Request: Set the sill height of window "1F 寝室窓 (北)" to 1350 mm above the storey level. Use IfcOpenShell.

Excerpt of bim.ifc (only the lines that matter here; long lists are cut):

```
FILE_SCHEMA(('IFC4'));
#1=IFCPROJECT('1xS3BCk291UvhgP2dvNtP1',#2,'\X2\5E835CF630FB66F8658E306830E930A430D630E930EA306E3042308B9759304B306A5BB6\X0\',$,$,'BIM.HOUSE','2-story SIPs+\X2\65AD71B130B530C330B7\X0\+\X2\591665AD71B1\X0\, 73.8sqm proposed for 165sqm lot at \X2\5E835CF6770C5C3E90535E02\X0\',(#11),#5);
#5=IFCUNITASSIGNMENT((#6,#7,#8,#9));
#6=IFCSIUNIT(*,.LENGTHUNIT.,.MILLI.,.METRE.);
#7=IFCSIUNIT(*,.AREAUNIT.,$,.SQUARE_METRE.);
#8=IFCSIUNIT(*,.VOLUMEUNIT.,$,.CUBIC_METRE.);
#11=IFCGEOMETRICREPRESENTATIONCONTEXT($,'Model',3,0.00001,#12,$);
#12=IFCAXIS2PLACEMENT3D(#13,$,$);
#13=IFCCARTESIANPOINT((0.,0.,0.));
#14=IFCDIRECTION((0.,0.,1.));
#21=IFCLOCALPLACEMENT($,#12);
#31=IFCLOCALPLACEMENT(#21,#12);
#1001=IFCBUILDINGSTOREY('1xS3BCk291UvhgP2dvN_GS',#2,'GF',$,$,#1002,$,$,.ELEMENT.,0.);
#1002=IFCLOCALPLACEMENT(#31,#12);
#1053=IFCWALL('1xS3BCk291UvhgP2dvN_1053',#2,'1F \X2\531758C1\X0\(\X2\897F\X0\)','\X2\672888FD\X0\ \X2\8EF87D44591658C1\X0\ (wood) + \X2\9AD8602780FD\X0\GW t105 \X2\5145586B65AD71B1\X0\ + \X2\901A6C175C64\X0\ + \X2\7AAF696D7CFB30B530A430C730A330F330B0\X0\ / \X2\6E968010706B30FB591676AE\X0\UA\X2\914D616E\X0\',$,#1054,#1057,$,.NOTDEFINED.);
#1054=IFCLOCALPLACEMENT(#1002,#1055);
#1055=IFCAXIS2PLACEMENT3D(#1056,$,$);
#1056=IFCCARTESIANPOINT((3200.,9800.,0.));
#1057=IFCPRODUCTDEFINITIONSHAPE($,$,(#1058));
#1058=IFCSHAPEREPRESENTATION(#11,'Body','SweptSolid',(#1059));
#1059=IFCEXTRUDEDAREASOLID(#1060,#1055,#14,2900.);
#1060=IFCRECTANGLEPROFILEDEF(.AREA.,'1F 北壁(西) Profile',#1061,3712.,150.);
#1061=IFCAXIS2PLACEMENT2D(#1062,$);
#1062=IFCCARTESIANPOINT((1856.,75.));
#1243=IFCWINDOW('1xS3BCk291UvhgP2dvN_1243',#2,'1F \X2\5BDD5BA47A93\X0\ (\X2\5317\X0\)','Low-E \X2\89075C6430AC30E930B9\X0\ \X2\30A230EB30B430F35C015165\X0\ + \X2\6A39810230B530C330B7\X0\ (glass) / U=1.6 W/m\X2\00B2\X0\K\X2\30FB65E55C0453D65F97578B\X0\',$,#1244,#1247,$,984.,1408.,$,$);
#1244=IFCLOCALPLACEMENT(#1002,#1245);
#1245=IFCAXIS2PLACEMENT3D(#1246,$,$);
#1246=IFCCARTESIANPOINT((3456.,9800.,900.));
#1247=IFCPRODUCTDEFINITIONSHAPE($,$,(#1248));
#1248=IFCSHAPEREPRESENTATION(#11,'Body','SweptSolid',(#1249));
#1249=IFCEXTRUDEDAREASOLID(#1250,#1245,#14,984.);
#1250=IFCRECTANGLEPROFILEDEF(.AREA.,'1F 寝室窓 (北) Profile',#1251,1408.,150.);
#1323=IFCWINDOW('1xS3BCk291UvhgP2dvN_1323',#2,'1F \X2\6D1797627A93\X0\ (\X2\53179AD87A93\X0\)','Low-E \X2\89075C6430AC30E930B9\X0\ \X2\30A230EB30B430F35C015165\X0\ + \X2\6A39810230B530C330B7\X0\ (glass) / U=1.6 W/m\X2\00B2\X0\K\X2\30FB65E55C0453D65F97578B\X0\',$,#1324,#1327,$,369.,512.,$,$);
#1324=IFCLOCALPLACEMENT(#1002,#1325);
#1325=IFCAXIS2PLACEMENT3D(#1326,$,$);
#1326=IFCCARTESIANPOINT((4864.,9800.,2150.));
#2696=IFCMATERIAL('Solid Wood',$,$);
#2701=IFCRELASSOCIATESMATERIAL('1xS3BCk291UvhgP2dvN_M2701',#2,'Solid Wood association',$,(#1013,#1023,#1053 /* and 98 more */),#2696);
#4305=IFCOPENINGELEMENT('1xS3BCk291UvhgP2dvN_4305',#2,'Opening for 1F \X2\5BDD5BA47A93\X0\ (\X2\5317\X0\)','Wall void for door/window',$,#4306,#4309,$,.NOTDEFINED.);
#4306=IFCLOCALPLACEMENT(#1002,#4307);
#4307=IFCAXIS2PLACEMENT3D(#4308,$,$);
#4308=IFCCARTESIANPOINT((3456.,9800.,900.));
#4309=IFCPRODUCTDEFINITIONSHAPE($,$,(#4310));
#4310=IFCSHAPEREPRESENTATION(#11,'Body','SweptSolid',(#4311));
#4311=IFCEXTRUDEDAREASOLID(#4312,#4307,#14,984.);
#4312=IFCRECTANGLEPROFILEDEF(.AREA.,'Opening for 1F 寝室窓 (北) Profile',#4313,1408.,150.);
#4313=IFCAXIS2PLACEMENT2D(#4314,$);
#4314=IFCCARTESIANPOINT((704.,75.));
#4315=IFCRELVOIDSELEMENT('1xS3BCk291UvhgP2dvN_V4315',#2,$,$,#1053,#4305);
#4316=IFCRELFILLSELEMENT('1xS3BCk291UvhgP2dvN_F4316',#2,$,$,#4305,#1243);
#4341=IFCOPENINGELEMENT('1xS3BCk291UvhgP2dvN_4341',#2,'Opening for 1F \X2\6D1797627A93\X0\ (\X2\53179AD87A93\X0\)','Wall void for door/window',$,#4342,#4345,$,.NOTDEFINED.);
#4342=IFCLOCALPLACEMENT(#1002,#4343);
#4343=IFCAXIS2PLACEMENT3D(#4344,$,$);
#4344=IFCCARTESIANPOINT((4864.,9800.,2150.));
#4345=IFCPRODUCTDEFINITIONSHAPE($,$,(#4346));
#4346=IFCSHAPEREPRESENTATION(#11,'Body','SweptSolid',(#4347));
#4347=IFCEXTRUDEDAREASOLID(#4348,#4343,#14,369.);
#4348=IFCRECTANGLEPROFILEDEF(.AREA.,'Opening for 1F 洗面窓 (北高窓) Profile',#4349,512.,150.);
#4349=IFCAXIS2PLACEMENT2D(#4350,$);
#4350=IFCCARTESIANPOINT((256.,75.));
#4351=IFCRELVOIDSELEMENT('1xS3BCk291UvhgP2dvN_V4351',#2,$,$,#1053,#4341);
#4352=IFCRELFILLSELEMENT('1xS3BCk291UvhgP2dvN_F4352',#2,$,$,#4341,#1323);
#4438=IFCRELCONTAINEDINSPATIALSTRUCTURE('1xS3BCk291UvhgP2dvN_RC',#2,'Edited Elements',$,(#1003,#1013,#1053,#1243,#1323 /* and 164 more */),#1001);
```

```python
import numpy as np
import ifcopenshell
import ifcopenshell.api.geometry
import ifcopenshell.geom
import ifcopenshell.util.element
import ifcopenshell.util.placement
import ifcopenshell.util.shape
import ifcopenshell.util.unit

model = ifcopenshell.open("bim.ifc")
unit_scale = ifcopenshell.util.unit.calculate_unit_scale(model)

window = model.by_guid("1xS3BCk291UvhgP2dvN_1243")
opening = window.FillsVoids[0].RelatingOpeningElement
storey = ifcopenshell.util.element.get_container(window, ifc_class="IfcBuildingStorey")
level = ifcopenshell.util.placement.get_local_placement(storey.ObjectPlacement)[2, 3]

# The opening's origin need not be at the sill, so measure its lowest point.
shape = ifcopenshell.geom.create_shape(ifcopenshell.geom.settings(), opening)
bottom = ifcopenshell.util.shape.get_shape_bottom_elevation(shape, shape.geometry) / unit_scale
dz = level + 1350.0 - bottom

shift = np.array([0.0, 0.0, dz])
# The window is not placed relative to its opening, so move both.
for product in (opening, window):
    matrix = ifcopenshell.util.placement.get_local_placement(product.ObjectPlacement)
    matrix[:3, 3] += shift
    ifcopenshell.api.geometry.edit_object_placement(model, product=product, matrix=matrix, is_si=False)

print(f"moved by {dz * unit_scale:+.3f} m")

model.write("bim_v2.ifc")
```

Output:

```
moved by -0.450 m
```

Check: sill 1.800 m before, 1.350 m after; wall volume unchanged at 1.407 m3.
